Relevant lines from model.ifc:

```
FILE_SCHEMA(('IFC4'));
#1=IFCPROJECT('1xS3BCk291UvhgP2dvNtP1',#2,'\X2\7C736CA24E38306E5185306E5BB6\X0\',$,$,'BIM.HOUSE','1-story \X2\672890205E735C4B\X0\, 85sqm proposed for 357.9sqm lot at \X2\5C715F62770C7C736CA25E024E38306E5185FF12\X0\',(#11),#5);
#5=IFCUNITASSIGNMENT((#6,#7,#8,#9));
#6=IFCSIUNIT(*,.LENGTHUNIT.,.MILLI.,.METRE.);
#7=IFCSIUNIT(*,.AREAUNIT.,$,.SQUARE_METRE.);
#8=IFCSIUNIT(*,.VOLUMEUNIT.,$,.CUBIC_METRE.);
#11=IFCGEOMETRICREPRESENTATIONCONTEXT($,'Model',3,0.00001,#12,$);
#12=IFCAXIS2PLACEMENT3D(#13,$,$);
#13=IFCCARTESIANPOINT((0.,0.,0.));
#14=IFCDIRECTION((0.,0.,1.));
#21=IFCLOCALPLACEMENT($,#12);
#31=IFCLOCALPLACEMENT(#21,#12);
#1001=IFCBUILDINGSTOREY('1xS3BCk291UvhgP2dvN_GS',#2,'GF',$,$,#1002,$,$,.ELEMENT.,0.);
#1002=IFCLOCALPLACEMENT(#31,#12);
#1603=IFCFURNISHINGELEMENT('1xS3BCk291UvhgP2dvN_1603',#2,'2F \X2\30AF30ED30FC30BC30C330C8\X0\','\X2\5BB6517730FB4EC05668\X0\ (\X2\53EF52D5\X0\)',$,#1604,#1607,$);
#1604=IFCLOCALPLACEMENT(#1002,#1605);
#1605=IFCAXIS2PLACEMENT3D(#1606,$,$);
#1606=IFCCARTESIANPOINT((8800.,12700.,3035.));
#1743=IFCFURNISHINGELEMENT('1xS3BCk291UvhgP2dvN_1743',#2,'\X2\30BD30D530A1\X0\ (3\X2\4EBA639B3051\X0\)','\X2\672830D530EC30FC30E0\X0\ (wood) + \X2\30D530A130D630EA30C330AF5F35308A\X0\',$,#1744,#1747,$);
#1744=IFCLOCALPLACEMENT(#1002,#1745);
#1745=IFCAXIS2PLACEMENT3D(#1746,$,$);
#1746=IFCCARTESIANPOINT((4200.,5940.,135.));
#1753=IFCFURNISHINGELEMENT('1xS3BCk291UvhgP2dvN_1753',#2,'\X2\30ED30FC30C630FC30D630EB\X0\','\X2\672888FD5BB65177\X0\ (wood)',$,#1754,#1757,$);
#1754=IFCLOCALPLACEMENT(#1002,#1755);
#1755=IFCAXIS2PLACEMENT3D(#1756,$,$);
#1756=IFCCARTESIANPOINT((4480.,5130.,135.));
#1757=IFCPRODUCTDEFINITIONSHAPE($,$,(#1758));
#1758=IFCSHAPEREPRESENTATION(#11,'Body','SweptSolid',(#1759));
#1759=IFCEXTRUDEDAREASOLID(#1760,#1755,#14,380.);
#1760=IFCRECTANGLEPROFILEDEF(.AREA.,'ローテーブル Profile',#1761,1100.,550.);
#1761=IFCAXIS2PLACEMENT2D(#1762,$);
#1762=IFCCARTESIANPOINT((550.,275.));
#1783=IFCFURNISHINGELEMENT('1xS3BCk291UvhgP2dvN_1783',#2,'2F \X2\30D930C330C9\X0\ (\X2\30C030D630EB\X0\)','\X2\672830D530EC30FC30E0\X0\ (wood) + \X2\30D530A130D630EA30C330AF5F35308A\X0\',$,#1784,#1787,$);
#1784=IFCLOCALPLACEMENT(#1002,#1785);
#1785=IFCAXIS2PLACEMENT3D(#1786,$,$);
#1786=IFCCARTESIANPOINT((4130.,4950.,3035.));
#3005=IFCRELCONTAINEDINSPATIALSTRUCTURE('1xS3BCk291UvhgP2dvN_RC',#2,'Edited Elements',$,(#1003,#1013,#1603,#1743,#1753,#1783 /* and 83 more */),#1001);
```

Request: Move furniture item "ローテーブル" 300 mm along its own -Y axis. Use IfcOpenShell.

```python
import ifcopenshell
import ifcopenshell.api.geometry
import ifcopenshell.util.placement
import ifcopenshell.util.unit

model = ifcopenshell.open("model.ifc")
unit_scale = ifcopenshell.util.unit.calculate_unit_scale(model)

item = model.by_guid("1xS3BCk291UvhgP2dvN_1753")
matrix = ifcopenshell.util.placement.get_local_placement(item.ObjectPlacement)
matrix[:3, 3] -= matrix[:3, 1] * 0.3 / unit_scale
ifcopenshell.api.geometry.edit_object_placement(model, product=item, matrix=matrix, is_si=False)

print(ifcopenshell.util.placement.get_local_placement(item.ObjectPlacement).round(3) + 0.0)

model.write("model_rev.ifc")
```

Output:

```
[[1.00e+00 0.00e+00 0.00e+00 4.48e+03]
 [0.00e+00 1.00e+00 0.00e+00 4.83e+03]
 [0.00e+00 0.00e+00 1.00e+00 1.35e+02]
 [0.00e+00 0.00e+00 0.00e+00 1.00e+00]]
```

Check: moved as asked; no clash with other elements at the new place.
